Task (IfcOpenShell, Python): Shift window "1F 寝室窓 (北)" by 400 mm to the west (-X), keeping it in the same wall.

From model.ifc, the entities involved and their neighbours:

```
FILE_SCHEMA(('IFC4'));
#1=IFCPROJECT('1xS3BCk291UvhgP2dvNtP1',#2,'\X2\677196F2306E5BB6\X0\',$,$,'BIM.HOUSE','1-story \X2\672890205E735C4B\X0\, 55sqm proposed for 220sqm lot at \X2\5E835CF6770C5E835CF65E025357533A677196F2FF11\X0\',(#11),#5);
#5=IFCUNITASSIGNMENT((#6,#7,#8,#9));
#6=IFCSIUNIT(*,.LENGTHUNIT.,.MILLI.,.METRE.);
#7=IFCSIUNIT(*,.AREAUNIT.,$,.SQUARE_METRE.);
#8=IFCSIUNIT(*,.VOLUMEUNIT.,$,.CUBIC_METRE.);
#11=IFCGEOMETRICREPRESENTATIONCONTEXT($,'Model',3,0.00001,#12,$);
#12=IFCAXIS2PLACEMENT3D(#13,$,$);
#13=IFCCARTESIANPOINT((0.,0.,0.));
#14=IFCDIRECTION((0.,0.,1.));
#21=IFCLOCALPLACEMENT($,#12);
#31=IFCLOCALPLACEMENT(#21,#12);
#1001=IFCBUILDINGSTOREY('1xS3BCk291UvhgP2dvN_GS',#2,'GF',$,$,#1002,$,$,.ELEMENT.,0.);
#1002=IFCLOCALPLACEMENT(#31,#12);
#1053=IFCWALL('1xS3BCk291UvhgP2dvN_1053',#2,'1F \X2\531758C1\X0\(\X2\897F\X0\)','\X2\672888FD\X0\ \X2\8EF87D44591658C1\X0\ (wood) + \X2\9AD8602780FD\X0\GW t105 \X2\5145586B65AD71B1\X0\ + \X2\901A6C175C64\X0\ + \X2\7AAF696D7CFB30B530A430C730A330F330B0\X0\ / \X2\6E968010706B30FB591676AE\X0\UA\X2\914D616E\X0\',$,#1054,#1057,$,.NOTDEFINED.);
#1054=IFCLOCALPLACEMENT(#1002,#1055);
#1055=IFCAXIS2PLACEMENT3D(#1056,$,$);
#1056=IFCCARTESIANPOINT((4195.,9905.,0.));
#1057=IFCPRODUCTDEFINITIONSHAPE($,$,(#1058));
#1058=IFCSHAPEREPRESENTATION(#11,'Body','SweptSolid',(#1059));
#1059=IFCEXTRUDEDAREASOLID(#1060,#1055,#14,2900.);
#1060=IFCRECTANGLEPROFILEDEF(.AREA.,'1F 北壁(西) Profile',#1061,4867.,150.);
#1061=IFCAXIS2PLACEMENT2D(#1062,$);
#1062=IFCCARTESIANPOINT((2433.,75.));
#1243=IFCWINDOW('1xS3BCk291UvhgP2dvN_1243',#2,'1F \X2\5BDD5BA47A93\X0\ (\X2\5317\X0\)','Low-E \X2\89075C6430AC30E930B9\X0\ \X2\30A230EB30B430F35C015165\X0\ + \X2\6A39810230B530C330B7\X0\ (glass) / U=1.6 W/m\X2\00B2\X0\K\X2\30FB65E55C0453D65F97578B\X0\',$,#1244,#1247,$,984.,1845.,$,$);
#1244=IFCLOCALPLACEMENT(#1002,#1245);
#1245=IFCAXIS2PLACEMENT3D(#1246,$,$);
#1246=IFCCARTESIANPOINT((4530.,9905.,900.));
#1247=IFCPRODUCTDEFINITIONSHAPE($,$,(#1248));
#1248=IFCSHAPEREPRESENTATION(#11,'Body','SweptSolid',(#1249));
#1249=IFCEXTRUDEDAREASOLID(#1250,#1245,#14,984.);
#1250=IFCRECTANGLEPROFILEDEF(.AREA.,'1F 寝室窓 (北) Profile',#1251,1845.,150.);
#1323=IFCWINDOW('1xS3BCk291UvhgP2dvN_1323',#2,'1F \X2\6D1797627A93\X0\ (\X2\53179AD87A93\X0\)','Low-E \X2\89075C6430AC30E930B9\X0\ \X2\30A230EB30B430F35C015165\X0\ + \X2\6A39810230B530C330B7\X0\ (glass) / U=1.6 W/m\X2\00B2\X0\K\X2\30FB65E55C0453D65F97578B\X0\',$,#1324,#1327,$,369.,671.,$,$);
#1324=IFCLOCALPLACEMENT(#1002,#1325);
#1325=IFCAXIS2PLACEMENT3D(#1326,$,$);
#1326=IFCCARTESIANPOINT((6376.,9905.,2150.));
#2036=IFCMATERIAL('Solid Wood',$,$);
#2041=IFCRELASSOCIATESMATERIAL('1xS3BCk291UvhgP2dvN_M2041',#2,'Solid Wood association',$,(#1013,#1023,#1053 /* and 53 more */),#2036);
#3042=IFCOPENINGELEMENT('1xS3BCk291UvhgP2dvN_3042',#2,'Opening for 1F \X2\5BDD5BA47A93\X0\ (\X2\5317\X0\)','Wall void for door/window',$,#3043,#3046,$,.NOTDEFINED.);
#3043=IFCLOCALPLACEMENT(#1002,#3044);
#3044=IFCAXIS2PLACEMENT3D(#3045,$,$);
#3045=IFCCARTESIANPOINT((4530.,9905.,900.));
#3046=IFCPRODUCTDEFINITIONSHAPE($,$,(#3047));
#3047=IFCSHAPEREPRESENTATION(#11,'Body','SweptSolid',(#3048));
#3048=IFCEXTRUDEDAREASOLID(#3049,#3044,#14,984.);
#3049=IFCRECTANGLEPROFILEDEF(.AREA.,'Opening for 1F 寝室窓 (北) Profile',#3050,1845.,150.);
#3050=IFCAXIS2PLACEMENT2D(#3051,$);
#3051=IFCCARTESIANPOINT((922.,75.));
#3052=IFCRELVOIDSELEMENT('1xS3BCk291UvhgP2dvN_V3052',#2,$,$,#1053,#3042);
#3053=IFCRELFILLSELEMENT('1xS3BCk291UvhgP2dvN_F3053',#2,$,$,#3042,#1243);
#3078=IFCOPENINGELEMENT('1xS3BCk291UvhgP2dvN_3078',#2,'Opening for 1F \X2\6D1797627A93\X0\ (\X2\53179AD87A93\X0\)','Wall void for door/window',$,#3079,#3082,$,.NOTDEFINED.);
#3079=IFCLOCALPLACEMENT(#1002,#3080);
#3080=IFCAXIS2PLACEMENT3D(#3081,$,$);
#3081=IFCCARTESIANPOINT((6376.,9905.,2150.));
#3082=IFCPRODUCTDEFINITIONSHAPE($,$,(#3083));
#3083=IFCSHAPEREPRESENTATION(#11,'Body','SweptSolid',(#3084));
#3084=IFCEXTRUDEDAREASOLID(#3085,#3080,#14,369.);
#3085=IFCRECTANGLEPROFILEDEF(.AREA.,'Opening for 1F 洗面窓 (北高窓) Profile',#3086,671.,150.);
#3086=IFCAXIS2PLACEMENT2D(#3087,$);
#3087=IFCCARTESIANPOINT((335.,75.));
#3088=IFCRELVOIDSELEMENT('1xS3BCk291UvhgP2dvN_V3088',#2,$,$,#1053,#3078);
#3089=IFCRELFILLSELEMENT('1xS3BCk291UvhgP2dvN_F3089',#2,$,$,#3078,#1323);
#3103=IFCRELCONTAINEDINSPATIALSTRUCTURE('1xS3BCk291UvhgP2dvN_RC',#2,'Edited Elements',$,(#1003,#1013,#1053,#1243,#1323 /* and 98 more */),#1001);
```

```python
import ifcopenshell
import ifcopenshell.api.geometry
import ifcopenshell.util.placement
import ifcopenshell.util.unit

model = ifcopenshell.open("model.ifc")
unit_scale = ifcopenshell.util.unit.calculate_unit_scale(model)

window = model.by_guid("1xS3BCk291UvhgP2dvN_1243")
opening = window.FillsVoids[0].RelatingOpeningElement
wall = opening.VoidsElements[0].RelatingBuildingElement

wall_matrix = ifcopenshell.util.placement.get_local_placement(wall.ObjectPlacement)
shift = wall_matrix[:3, 0] * -0.4 / unit_scale
before = ifcopenshell.util.placement.get_local_placement(window.ObjectPlacement)[:3, 3].copy()

# The window is not placed relative to its opening, so move both.
for product in (opening, window):
    matrix = ifcopenshell.util.placement.get_local_placement(product.ObjectPlacement)
    matrix[:3, 3] += shift
    ifcopenshell.api.geometry.edit_object_placement(model, product=product, matrix=matrix, is_si=False)

after = ifcopenshell.util.placement.get_local_placement(window.ObjectPlacement)[:3, 3]
print("window moved by", (after - before).round(3) + 0.0)

model.write("model_rev.ifc")
```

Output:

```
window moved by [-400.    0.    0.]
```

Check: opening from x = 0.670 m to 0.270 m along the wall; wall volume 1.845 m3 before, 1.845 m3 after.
